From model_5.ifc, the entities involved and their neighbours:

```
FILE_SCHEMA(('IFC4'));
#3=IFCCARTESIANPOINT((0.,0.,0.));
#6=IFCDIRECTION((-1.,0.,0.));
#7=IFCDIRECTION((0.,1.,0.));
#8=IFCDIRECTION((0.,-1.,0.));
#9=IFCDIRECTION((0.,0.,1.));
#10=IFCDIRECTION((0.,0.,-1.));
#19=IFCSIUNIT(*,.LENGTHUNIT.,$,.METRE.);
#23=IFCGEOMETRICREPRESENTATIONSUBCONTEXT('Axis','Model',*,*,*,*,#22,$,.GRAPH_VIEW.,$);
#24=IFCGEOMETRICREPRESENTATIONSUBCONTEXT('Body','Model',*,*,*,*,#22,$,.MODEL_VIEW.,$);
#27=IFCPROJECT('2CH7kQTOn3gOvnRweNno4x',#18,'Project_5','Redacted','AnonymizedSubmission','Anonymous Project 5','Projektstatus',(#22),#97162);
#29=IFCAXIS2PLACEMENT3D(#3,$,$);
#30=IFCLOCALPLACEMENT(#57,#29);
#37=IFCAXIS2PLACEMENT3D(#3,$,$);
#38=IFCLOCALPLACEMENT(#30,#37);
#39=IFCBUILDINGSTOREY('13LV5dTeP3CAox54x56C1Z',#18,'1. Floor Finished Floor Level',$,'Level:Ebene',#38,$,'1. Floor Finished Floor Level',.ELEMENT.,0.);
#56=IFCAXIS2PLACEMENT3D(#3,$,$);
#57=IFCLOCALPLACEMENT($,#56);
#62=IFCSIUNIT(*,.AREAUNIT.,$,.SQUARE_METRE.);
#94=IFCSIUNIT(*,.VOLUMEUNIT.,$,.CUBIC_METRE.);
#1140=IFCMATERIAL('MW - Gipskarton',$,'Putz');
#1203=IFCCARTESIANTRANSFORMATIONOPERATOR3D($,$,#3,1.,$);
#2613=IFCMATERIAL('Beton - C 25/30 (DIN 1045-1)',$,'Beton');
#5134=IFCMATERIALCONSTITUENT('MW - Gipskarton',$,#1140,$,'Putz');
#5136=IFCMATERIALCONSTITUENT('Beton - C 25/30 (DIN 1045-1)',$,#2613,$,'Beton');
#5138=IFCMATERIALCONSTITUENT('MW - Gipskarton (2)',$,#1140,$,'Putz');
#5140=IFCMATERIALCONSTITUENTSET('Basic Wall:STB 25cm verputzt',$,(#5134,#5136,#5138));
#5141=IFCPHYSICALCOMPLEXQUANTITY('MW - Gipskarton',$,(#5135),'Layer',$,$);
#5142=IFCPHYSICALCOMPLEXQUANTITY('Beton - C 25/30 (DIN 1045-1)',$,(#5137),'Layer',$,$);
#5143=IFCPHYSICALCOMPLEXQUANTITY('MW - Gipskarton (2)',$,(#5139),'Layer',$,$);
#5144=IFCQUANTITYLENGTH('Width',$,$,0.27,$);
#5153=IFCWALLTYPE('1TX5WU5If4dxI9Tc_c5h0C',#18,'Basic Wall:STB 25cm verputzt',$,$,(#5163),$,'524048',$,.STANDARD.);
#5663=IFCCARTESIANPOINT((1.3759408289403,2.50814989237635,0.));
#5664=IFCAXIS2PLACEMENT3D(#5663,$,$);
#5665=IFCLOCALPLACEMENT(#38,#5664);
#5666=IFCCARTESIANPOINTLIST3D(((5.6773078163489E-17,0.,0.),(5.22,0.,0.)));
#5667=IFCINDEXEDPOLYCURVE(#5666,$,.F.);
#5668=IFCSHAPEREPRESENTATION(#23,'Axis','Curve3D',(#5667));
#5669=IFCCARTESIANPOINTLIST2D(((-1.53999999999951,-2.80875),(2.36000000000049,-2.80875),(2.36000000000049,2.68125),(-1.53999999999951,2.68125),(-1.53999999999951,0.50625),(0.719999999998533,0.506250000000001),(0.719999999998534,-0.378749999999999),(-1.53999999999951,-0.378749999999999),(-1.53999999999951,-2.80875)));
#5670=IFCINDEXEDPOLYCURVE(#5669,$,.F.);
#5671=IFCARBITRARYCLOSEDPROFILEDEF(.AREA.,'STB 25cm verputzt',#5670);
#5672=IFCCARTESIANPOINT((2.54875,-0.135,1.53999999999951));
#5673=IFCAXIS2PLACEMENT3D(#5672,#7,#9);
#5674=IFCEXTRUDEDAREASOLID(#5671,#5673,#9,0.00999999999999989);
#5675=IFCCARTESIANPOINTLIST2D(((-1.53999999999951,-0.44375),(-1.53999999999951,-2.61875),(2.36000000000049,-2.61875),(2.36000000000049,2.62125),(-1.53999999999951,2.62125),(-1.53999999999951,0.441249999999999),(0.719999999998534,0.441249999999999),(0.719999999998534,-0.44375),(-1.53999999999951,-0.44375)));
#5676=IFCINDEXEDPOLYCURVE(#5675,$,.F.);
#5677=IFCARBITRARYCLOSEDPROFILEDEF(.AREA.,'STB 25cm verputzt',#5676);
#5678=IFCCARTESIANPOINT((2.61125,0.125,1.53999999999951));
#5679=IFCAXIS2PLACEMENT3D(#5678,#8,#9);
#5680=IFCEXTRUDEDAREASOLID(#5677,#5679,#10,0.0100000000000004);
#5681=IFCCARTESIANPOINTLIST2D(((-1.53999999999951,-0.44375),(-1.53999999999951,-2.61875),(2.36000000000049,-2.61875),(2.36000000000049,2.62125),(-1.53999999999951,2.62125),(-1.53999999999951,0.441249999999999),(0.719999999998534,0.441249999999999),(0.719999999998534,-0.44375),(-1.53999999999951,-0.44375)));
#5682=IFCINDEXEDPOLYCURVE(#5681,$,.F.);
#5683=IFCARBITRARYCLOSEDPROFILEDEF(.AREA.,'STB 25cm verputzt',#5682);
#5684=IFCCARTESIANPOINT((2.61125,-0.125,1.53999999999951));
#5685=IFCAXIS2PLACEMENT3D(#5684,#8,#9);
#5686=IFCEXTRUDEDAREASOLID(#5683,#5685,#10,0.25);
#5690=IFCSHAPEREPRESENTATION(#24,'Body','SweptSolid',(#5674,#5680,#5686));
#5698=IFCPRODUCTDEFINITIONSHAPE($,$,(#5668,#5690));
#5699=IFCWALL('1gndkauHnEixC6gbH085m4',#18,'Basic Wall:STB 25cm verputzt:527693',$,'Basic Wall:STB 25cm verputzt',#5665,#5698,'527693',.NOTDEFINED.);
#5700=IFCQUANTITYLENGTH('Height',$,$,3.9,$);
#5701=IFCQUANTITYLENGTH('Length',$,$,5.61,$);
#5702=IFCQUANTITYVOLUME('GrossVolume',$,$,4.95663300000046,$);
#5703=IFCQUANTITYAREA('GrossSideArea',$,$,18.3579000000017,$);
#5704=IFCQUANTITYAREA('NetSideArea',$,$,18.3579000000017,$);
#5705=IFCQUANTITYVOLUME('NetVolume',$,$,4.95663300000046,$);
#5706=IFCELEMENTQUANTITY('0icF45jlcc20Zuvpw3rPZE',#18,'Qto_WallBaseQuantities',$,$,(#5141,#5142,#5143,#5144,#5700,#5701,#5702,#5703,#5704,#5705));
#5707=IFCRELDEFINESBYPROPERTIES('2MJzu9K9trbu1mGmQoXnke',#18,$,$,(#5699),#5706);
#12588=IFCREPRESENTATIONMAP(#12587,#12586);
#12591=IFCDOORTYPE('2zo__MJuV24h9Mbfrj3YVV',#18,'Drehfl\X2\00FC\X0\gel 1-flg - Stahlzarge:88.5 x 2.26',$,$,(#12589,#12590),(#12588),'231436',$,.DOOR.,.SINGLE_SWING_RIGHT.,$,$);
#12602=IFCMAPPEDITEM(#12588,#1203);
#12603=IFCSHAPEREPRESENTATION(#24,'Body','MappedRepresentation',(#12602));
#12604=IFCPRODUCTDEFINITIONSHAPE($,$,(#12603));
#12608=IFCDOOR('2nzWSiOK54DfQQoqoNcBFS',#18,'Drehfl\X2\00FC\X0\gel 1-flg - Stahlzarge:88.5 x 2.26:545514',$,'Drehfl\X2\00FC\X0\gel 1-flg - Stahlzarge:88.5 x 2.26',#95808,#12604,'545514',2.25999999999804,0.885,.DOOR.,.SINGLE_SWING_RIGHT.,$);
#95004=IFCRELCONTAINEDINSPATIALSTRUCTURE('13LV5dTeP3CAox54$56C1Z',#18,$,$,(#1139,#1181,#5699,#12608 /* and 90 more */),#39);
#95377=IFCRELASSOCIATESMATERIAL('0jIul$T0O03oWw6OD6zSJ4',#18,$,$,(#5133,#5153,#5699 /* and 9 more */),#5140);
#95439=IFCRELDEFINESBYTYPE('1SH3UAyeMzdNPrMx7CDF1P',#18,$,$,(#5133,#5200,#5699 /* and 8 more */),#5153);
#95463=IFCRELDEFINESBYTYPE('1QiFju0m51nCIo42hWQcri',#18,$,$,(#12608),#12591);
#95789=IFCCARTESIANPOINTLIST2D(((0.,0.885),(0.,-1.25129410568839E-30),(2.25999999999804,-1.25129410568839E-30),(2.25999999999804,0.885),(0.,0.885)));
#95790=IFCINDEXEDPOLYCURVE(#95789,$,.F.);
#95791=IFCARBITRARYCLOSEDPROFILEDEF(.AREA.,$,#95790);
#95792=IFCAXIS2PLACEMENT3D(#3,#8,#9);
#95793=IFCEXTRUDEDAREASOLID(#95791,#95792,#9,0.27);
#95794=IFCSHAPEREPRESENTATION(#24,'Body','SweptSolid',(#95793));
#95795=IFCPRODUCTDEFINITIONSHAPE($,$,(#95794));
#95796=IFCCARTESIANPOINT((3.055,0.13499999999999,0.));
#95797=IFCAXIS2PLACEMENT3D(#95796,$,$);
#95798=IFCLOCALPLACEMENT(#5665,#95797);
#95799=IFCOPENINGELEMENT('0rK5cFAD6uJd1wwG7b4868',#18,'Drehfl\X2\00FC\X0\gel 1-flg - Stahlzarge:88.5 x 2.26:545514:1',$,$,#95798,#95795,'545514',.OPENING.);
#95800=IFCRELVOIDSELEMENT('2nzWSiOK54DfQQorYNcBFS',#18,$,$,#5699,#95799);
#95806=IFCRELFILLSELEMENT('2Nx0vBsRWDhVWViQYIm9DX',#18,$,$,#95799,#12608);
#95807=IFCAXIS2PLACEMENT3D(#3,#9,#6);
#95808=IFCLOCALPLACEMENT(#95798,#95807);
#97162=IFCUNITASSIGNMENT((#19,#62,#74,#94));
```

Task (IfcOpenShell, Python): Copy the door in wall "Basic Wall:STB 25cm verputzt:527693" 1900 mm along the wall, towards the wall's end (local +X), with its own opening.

```python
import ifcopenshell
import ifcopenshell.api.feature
import ifcopenshell.api.geometry
import ifcopenshell.api.pset
import ifcopenshell.api.root
import ifcopenshell.geom
import ifcopenshell.util.element
import ifcopenshell.util.placement
import ifcopenshell.util.shape
import ifcopenshell.util.unit

model = ifcopenshell.open("model_5.ifc")
unit_scale = ifcopenshell.util.unit.calculate_unit_scale(model)
area_scale = ifcopenshell.util.unit.calculate_unit_scale(model, "AREAUNIT")
volume_scale = ifcopenshell.util.unit.calculate_unit_scale(model, "VOLUMEUNIT")
settings = ifcopenshell.geom.settings()


def volume(element):
    """Net volume in cubic metres, openings subtracted."""
    shape = ifcopenshell.geom.create_shape(settings, element)
    return ifcopenshell.util.shape.get_volume(shape.geometry)


def reuse_history(source, copy):
    """copy_class also copies each property set's owner history, people and application; keep the originals."""
    for rel in copy.IsDefinedBy:
        if rel.is_a("IfcRelDefinesByProperties") and (history := rel.RelatingPropertyDefinition.OwnerHistory):
            rel.RelatingPropertyDefinition.OwnerHistory = source.OwnerHistory
            ifcopenshell.util.element.remove_deep2(model, history)


door = model.by_guid("2nzWSiOK54DfQQoqoNcBFS")
opening = door.FillsVoids[0].RelatingOpeningElement
wall = opening.VoidsElements[0].RelatingBuildingElement
before = volume(wall)
shift = ifcopenshell.util.placement.get_local_placement(wall.ObjectPlacement)[:3, 0] * 1.9 / unit_scale

# copy_class copies the void relationship, type, container and properties, but no geometry.
new_opening = ifcopenshell.api.root.copy_class(model, product=opening)
new_opening.Representation = ifcopenshell.util.element.copy_deep(
    model, opening.Representation, exclude=["IfcGeometricRepresentationContext", "IfcRepresentationMap"]
)
new_opening.Name = "Drehflügel 1-flg - Stahlzarge:88.5 x 2.26"
new_opening.Tag = None
reuse_history(opening, new_opening)
new_door = ifcopenshell.api.root.copy_class(model, product=door)
new_door.Representation = ifcopenshell.util.element.copy_deep(
    model, door.Representation, exclude=["IfcGeometricRepresentationContext", "IfcRepresentationMap"]
)
new_door.Name = "Drehflügel 1-flg - Stahlzarge:88.5 x 2.26"
new_door.Tag = None
reuse_history(door, new_door)
ifcopenshell.api.feature.add_filling(model, opening=new_opening, element=new_door)

for old, new in ((opening, new_opening), (door, new_door)):
    matrix = ifcopenshell.util.placement.get_local_placement(old.ObjectPlacement)
    matrix[:3, 3] += shift
    ifcopenshell.api.geometry.edit_object_placement(model, product=new, matrix=matrix, is_si=False)

after = volume(wall)
thickness = 0.27  # wall thickness in metres

# Update the wall's stored quantities.
qto = model.by_id(ifcopenshell.util.element.get_pset(wall, "Qto_WallBaseQuantities", should_inherit=False)["id"])
ifcopenshell.api.pset.edit_qto(model, qto=qto, properties={
    "NetSideArea": after / thickness / area_scale,
    "NetVolume": after / volume_scale,
})

print(f"wall volume {before:.3f} -> {after:.3f} m3")

model.write("model_5_rev.ifc")
```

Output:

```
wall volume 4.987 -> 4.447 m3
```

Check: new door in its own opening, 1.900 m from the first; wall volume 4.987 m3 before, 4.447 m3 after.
